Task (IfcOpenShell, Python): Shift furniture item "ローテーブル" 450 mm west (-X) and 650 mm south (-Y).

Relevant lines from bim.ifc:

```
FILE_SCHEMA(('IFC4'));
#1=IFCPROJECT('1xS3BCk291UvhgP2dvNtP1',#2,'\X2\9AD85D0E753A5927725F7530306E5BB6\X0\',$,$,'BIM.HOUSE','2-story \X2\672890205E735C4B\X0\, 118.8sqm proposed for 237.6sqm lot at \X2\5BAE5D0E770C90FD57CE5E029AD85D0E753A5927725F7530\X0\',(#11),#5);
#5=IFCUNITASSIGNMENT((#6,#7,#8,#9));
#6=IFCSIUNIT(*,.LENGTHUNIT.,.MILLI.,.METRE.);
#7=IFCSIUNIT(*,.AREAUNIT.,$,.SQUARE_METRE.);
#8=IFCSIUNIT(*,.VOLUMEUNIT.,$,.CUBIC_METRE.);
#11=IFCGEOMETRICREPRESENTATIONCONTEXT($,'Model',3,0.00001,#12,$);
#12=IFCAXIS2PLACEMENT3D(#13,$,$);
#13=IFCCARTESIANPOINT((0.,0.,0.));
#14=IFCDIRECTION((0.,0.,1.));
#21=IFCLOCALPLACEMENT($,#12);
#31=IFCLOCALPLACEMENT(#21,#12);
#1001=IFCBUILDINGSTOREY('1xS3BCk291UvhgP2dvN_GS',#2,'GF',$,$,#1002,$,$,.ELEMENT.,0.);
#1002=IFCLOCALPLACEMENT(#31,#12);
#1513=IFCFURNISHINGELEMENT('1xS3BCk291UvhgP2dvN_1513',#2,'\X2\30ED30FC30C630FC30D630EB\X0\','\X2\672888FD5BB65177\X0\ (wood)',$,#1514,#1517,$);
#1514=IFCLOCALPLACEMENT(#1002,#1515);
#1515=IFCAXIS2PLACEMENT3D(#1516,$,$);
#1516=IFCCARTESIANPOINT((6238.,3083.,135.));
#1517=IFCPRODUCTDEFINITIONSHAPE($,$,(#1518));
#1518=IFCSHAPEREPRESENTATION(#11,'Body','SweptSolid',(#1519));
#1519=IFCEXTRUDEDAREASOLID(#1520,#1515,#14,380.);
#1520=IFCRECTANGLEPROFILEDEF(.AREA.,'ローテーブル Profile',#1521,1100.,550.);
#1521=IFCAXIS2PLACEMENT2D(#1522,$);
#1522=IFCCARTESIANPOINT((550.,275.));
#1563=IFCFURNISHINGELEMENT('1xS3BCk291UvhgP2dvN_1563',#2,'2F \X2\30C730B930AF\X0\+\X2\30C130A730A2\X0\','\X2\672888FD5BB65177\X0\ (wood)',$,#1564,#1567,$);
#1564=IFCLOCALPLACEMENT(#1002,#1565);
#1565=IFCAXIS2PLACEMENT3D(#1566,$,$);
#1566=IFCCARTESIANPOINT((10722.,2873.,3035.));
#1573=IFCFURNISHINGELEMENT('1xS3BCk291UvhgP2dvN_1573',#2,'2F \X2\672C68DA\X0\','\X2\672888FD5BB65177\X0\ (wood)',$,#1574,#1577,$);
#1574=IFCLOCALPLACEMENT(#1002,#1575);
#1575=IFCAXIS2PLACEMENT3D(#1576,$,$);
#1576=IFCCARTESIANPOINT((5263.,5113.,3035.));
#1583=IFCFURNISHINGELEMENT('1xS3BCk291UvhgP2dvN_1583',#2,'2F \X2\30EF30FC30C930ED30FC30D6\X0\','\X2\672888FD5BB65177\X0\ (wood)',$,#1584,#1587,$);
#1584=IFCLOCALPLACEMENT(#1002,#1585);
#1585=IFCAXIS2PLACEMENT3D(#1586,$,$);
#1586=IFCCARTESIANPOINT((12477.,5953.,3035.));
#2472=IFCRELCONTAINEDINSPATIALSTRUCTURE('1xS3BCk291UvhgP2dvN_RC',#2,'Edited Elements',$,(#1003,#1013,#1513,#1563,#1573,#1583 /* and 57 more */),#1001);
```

```python
import ifcopenshell
import ifcopenshell.api.geometry
import ifcopenshell.util.placement
import ifcopenshell.util.unit

model = ifcopenshell.open("bim.ifc")
unit_scale = ifcopenshell.util.unit.calculate_unit_scale(model)

item = model.by_id(1513)
matrix = ifcopenshell.util.placement.get_local_placement(item.ObjectPlacement)
matrix[0, 3] -= 0.45 / unit_scale
matrix[1, 3] -= 0.65 / unit_scale
ifcopenshell.api.geometry.edit_object_placement(model, product=item, matrix=matrix, is_si=False)

print(ifcopenshell.util.placement.get_local_placement(item.ObjectPlacement).round(3) + 0.0)

model.write("bim-out.ifc")
```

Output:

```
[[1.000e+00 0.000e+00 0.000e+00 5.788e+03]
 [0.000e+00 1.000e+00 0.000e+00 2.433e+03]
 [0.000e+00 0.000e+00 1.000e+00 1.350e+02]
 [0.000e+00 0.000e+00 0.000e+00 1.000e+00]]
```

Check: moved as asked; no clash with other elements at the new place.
